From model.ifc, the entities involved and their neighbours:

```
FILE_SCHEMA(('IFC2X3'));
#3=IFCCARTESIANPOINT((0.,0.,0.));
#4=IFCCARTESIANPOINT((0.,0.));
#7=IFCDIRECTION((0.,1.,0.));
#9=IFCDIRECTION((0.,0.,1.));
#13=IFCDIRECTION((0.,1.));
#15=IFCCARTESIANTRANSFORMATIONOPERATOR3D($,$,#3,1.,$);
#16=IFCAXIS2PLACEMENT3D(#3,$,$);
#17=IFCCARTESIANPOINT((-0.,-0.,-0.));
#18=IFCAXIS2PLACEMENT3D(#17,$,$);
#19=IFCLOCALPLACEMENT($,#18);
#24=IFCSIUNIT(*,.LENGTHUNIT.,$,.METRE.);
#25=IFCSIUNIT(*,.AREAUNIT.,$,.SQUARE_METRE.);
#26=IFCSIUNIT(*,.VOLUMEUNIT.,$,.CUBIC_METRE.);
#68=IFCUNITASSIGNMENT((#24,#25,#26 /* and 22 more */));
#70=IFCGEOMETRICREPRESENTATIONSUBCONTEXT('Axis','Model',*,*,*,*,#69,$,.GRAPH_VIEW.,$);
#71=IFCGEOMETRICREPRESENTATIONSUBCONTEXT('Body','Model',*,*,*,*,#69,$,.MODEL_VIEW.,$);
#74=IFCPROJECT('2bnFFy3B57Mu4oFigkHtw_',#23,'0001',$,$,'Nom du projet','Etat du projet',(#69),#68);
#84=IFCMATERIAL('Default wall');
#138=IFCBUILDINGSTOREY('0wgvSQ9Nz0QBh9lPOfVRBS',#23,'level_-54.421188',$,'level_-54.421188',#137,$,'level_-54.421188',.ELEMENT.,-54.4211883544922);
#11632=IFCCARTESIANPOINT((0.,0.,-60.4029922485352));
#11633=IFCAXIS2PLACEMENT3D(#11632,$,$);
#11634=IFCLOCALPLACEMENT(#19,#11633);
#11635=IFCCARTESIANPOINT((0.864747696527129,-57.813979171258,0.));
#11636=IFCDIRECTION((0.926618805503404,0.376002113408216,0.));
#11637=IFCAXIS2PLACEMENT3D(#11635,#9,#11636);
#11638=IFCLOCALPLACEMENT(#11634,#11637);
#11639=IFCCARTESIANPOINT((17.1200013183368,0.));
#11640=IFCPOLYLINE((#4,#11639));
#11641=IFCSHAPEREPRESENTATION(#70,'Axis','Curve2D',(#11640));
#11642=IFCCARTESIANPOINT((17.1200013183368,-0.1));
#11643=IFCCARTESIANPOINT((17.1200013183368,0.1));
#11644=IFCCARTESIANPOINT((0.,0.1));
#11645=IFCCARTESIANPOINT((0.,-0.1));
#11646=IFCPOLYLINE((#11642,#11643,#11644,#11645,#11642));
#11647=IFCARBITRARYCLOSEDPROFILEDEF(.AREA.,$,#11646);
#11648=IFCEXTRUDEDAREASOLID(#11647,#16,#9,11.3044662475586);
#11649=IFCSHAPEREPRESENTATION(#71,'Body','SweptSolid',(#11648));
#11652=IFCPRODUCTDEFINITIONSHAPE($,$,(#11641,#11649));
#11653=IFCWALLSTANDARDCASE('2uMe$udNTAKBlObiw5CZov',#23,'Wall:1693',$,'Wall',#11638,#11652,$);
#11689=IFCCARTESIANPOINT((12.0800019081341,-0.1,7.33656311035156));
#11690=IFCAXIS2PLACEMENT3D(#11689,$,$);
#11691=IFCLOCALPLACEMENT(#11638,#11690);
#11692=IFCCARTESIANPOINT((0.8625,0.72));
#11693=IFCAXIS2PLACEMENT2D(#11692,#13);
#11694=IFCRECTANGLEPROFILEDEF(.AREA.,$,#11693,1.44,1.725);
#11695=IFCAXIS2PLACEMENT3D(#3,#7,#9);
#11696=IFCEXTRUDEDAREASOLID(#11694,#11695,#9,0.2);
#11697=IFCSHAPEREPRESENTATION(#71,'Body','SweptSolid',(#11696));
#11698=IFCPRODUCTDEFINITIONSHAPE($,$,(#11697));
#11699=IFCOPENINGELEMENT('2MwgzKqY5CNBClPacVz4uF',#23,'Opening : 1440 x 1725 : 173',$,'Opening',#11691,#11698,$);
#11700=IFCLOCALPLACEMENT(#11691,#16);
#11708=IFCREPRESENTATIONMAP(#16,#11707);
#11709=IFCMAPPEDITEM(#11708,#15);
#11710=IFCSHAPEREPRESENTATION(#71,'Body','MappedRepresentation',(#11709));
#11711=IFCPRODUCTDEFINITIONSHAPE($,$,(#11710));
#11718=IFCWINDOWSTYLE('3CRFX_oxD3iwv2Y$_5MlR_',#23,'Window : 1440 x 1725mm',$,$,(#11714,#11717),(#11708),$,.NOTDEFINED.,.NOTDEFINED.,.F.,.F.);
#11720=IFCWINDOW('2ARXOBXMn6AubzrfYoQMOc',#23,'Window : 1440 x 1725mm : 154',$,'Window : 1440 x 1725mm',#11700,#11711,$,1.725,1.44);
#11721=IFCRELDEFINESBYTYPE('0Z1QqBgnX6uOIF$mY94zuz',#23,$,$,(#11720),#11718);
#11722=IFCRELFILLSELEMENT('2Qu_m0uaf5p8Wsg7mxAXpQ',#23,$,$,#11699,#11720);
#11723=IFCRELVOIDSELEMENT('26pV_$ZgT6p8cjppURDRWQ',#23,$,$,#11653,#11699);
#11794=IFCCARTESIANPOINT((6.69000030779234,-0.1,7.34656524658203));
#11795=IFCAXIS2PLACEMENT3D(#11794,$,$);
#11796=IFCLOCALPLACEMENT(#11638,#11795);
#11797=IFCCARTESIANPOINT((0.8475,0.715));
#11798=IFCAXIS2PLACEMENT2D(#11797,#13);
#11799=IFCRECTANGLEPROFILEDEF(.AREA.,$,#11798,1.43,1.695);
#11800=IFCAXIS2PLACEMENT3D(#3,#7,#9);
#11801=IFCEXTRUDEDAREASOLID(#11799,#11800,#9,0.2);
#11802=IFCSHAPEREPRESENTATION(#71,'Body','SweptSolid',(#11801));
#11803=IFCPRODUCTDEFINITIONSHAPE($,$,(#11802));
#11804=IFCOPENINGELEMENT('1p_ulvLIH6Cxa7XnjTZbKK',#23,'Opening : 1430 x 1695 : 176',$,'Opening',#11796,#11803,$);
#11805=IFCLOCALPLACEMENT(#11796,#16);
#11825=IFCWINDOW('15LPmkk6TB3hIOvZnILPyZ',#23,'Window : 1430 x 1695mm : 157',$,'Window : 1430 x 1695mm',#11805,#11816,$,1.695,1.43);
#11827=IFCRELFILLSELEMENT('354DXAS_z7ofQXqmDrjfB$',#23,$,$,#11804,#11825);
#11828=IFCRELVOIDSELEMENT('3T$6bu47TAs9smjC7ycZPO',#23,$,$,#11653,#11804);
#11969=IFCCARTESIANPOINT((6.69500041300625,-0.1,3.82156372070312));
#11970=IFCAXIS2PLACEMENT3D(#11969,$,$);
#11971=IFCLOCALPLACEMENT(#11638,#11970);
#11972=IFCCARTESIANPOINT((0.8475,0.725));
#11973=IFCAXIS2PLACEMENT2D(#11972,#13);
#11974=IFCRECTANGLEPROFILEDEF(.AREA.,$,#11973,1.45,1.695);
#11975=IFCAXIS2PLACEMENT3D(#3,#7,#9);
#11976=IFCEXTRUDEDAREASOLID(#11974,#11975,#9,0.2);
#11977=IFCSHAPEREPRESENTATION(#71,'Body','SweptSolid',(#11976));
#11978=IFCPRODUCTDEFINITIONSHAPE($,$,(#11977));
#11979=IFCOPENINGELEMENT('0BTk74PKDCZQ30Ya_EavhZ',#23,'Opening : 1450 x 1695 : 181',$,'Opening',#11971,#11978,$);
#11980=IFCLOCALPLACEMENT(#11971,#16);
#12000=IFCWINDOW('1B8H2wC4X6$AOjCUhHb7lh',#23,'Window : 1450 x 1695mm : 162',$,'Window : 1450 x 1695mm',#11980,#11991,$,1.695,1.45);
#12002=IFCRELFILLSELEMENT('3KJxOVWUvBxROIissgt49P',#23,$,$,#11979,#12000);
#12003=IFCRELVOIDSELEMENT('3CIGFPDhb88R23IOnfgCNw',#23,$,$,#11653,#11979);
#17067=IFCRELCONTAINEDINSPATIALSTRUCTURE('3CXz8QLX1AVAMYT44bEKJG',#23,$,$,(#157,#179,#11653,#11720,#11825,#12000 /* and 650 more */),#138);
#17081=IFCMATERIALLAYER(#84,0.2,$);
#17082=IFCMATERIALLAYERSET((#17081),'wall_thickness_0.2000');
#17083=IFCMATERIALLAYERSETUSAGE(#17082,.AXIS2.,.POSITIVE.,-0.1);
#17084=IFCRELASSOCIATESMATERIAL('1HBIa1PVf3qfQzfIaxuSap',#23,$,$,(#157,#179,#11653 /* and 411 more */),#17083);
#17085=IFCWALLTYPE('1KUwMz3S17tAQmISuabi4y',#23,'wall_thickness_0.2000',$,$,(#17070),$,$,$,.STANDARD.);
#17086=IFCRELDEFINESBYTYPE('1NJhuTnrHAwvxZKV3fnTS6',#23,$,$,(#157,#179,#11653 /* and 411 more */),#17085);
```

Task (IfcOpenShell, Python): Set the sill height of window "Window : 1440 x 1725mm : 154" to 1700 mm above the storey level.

```python
import numpy as np
import ifcopenshell
import ifcopenshell.api.geometry
import ifcopenshell.geom
import ifcopenshell.util.element
import ifcopenshell.util.placement
import ifcopenshell.util.shape
import ifcopenshell.util.unit

model = ifcopenshell.open("model.ifc")
unit_scale = ifcopenshell.util.unit.calculate_unit_scale(model)

window = model.by_id(11720)
opening = window.FillsVoids[0].RelatingOpeningElement
storey = ifcopenshell.util.element.get_container(window, ifc_class="IfcBuildingStorey")
level = ifcopenshell.util.placement.get_local_placement(storey.ObjectPlacement)[2, 3]

# The opening's origin need not be at the sill, so measure its lowest point.
shape = ifcopenshell.geom.create_shape(ifcopenshell.geom.settings(), opening)
bottom = ifcopenshell.util.shape.get_shape_bottom_elevation(shape, shape.geometry) / unit_scale
dz = level + 1.7 / unit_scale - bottom

shift = np.array([0.0, 0.0, dz])
# The window is placed relative to its opening, so it follows when the opening moves.
matrix = ifcopenshell.util.placement.get_local_placement(opening.ObjectPlacement)
matrix[:3, 3] += shift
ifcopenshell.api.geometry.edit_object_placement(
    model, product=opening, matrix=matrix, is_si=False, should_transform_children=True
)

print(f"moved by {dz * unit_scale:+.3f} m")

model.write("model_v2.ifc")
```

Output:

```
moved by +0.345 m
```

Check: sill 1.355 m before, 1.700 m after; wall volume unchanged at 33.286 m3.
